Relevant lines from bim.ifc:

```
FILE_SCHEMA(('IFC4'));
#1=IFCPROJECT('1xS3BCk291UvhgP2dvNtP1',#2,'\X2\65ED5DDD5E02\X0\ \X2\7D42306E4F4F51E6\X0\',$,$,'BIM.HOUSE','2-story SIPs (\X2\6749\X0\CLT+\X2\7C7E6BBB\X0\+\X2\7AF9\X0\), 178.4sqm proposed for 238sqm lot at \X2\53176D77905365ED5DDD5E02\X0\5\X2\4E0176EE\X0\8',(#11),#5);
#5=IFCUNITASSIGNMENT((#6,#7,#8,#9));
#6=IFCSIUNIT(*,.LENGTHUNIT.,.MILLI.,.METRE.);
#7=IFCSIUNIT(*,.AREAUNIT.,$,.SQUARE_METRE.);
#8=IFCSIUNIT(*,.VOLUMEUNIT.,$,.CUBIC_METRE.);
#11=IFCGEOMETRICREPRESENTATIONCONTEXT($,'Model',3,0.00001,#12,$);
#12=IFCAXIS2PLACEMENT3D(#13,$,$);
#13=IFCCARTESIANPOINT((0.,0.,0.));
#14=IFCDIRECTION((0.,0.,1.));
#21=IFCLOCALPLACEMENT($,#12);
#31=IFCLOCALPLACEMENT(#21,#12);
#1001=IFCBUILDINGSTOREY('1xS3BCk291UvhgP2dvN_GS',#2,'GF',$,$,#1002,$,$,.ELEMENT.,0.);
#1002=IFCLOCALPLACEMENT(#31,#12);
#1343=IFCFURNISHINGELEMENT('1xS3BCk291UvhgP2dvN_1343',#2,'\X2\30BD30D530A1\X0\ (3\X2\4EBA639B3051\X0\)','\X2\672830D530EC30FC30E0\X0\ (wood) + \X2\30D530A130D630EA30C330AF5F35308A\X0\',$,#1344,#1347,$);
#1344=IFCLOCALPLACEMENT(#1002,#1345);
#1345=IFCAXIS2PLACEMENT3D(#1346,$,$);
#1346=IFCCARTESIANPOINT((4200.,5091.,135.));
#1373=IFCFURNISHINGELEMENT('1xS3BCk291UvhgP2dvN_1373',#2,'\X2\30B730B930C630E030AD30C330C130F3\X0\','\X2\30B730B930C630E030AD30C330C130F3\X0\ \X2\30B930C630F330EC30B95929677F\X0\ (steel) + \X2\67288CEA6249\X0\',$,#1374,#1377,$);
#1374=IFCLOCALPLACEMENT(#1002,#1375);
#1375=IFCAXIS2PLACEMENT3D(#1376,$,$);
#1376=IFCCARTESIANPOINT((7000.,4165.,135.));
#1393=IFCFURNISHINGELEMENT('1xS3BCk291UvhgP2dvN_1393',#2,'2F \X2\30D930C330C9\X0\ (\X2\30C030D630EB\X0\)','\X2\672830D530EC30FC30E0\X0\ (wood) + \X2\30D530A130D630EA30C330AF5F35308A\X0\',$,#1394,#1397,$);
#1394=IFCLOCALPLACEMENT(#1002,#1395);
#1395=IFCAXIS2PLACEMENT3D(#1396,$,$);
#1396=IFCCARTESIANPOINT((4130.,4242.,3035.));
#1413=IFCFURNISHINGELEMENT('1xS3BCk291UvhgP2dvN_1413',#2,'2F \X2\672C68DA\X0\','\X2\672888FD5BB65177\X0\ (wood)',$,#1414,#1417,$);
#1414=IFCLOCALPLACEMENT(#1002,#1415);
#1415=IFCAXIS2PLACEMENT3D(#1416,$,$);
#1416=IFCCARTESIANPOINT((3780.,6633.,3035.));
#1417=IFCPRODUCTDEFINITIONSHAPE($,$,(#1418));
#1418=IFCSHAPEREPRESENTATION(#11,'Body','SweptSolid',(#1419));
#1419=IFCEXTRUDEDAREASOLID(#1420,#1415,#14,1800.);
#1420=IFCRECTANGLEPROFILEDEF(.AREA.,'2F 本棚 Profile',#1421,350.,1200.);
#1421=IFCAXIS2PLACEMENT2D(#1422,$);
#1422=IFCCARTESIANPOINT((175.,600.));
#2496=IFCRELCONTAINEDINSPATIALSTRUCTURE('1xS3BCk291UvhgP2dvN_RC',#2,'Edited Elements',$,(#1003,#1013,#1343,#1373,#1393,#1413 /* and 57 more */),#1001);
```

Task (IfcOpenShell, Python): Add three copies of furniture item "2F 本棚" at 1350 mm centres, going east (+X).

```python
import numpy as np
import ifcopenshell
import ifcopenshell.api.geometry
import ifcopenshell.api.root
import ifcopenshell.util.element
import ifcopenshell.util.placement
import ifcopenshell.util.unit

model = ifcopenshell.open("bim.ifc")
unit_scale = ifcopenshell.util.unit.calculate_unit_scale(model)


def reuse_history(source, copy):
    """copy_class also copies each property set's owner history, people and application; keep the originals."""
    for rel in copy.IsDefinedBy:
        if rel.is_a("IfcRelDefinesByProperties") and (history := rel.RelatingPropertyDefinition.OwnerHistory):
            rel.RelatingPropertyDefinition.OwnerHistory = source.OwnerHistory
            ifcopenshell.util.element.remove_deep2(model, history)


source = model.by_guid("1xS3BCk291UvhgP2dvN_1413")
base = ifcopenshell.util.placement.get_local_placement(source.ObjectPlacement)
step = np.array([1.0, 0.0, 0.0]) * 1.35 / unit_scale

for i in range(1, 4):
    copy = ifcopenshell.api.root.copy_class(model, product=source)
    copy.Representation = ifcopenshell.util.element.copy_deep(
        model, source.Representation, exclude=["IfcGeometricRepresentationContext", "IfcRepresentationMap"]
    )
    reuse_history(source, copy)
    matrix = base.copy()
    matrix[:3, 3] += i * step
    print("added at", matrix[:3, 3].round(3) + 0.0)
    ifcopenshell.api.geometry.edit_object_placement(model, product=copy, matrix=matrix, is_si=False)

model.write("bim_rev.ifc")
```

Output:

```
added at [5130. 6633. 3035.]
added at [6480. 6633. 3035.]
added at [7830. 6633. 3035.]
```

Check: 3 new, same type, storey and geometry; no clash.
